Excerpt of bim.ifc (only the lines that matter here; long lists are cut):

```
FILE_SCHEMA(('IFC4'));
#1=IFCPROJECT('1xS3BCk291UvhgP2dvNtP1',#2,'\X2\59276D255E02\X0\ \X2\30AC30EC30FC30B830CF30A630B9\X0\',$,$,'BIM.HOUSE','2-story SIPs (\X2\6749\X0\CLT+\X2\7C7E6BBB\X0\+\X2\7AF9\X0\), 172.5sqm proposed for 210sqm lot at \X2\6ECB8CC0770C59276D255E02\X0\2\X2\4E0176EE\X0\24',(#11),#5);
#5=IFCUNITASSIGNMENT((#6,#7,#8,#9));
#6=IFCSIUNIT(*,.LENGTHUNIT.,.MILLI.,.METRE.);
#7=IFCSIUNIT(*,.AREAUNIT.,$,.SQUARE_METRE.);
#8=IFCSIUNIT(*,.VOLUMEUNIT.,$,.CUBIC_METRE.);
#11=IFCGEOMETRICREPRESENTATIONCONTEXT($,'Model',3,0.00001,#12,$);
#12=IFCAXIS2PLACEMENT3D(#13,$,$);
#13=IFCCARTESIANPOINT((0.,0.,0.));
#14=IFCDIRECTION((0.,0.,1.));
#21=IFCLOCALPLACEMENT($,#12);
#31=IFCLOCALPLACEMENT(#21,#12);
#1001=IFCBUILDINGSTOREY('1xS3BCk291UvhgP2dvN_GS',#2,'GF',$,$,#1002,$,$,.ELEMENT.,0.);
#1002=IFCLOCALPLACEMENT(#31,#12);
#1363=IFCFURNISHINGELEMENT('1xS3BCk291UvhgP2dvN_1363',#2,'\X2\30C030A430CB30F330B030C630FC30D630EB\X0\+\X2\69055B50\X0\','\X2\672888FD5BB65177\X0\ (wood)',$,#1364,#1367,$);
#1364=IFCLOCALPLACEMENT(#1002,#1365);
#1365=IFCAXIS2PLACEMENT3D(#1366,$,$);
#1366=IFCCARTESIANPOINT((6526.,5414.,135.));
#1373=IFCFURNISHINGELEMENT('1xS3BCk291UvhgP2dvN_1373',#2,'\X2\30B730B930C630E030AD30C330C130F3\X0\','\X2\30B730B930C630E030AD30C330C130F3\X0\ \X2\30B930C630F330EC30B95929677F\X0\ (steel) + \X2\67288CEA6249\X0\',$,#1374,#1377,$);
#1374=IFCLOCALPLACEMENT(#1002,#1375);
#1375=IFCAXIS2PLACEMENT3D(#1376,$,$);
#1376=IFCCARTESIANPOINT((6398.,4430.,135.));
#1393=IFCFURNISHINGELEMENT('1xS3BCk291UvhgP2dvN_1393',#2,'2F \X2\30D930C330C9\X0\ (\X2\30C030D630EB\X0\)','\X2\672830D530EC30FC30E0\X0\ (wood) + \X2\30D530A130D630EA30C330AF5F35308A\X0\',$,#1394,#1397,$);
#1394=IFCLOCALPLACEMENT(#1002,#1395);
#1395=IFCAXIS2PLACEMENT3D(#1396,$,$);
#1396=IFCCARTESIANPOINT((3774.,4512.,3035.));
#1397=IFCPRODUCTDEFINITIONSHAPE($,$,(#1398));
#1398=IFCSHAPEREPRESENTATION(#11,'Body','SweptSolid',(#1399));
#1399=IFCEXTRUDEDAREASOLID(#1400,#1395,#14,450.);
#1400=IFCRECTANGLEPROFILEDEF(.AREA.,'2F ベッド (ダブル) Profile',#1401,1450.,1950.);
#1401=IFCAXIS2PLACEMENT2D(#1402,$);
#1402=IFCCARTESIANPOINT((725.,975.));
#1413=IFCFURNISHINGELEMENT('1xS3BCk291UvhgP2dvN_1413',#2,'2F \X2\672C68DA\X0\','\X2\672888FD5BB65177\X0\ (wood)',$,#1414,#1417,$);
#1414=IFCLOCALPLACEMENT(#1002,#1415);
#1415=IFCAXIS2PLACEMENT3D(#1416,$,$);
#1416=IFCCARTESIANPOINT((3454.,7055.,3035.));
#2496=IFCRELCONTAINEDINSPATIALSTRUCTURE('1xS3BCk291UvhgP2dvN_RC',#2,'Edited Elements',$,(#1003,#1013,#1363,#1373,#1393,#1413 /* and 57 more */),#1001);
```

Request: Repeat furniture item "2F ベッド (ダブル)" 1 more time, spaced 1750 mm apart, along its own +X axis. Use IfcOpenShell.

```python
import ifcopenshell
import ifcopenshell.api.geometry
import ifcopenshell.api.root
import ifcopenshell.util.element
import ifcopenshell.util.placement
import ifcopenshell.util.unit

model = ifcopenshell.open("bim.ifc")
unit_scale = ifcopenshell.util.unit.calculate_unit_scale(model)


def reuse_history(source, copy):
    """copy_class also copies each property set's owner history, people and application; keep the originals."""
    for rel in copy.IsDefinedBy:
        if rel.is_a("IfcRelDefinesByProperties") and (history := rel.RelatingPropertyDefinition.OwnerHistory):
            rel.RelatingPropertyDefinition.OwnerHistory = source.OwnerHistory
            ifcopenshell.util.element.remove_deep2(model, history)


source = model.by_id(1393)
base = ifcopenshell.util.placement.get_local_placement(source.ObjectPlacement)
step = base[:3, 0] * 1.75 / unit_scale

for i in range(1, 2):
    copy = ifcopenshell.api.root.copy_class(model, product=source)
    copy.Representation = ifcopenshell.util.element.copy_deep(
        model, source.Representation, exclude=["IfcGeometricRepresentationContext", "IfcRepresentationMap"]
    )
    reuse_history(source, copy)
    matrix = base.copy()
    matrix[:3, 3] += i * step
    print("added at", matrix[:3, 3].round(3) + 0.0)
    ifcopenshell.api.geometry.edit_object_placement(model, product=copy, matrix=matrix, is_si=False)

model.write("bim_rev.ifc")
```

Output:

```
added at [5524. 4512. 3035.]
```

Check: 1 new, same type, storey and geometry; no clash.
